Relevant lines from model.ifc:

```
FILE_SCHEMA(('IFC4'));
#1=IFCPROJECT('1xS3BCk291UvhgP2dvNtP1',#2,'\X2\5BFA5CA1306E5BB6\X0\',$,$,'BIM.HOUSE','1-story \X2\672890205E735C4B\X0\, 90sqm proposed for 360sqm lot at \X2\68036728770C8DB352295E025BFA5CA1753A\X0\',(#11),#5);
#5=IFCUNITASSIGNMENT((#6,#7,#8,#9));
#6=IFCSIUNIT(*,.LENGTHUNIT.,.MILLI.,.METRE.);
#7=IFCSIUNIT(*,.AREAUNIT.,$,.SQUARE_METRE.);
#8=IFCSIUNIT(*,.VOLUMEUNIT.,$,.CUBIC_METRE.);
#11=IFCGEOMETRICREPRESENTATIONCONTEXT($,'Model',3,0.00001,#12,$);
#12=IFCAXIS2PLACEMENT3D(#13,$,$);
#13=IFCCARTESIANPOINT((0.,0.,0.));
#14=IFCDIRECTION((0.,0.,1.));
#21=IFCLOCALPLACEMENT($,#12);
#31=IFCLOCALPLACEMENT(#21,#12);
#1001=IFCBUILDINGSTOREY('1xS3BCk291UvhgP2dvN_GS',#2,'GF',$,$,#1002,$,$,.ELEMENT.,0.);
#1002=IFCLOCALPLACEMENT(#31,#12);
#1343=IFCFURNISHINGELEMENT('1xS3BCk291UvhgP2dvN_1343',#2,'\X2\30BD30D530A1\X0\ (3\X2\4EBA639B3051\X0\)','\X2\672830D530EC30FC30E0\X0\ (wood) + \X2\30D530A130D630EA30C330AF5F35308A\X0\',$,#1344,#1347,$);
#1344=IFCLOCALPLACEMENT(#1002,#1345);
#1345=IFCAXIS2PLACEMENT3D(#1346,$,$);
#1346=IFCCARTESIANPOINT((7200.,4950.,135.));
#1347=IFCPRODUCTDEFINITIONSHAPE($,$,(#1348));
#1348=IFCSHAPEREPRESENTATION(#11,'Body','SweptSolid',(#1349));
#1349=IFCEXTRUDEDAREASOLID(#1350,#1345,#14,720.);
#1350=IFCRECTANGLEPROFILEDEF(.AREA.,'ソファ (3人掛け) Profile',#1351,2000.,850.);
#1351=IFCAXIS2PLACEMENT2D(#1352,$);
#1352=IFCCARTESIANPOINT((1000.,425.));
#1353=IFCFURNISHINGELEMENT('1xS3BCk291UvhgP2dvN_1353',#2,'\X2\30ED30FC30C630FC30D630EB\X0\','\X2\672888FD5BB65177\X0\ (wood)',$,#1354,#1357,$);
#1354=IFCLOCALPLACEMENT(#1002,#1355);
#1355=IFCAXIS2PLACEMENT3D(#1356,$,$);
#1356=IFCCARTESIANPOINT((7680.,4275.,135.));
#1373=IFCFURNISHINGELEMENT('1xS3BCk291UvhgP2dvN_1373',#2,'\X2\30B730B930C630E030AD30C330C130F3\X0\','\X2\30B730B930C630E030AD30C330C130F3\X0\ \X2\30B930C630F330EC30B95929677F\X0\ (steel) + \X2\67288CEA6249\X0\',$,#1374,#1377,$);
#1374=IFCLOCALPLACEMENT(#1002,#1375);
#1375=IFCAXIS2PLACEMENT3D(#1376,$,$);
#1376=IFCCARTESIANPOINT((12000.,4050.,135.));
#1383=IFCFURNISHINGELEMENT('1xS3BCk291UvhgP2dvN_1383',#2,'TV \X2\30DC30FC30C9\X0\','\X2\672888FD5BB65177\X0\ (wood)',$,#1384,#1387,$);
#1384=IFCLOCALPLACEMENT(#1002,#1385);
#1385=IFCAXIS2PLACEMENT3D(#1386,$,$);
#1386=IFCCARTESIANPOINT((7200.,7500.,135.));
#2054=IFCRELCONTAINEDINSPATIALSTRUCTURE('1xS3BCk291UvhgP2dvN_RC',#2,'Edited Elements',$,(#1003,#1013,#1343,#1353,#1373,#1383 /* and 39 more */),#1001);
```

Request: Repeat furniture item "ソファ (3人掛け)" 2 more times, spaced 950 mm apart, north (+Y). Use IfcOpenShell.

```python
import numpy as np
import ifcopenshell
import ifcopenshell.api.geometry
import ifcopenshell.api.root
import ifcopenshell.util.element
import ifcopenshell.util.placement
import ifcopenshell.util.unit

model = ifcopenshell.open("model.ifc")
unit_scale = ifcopenshell.util.unit.calculate_unit_scale(model)


def reuse_history(source, copy):
    """copy_class also copies each property set's owner history, people and application; keep the originals."""
    for rel in copy.IsDefinedBy:
        if rel.is_a("IfcRelDefinesByProperties") and (history := rel.RelatingPropertyDefinition.OwnerHistory):
            rel.RelatingPropertyDefinition.OwnerHistory = source.OwnerHistory
            ifcopenshell.util.element.remove_deep2(model, history)


source = model.by_id(1343)
base = ifcopenshell.util.placement.get_local_placement(source.ObjectPlacement)
step = np.array([0.0, 1.0, 0.0]) * 0.95 / unit_scale

for i in range(1, 3):
    copy = ifcopenshell.api.root.copy_class(model, product=source)
    copy.Representation = ifcopenshell.util.element.copy_deep(
        model, source.Representation, exclude=["IfcGeometricRepresentationContext", "IfcRepresentationMap"]
    )
    reuse_history(source, copy)
    matrix = base.copy()
    matrix[:3, 3] += i * step
    print("added at", matrix[:3, 3].round(3) + 0.0)
    ifcopenshell.api.geometry.edit_object_placement(model, product=copy, matrix=matrix, is_si=False)

model.write("model_rev.ifc")
```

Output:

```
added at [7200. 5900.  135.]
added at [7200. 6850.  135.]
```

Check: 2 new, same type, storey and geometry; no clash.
